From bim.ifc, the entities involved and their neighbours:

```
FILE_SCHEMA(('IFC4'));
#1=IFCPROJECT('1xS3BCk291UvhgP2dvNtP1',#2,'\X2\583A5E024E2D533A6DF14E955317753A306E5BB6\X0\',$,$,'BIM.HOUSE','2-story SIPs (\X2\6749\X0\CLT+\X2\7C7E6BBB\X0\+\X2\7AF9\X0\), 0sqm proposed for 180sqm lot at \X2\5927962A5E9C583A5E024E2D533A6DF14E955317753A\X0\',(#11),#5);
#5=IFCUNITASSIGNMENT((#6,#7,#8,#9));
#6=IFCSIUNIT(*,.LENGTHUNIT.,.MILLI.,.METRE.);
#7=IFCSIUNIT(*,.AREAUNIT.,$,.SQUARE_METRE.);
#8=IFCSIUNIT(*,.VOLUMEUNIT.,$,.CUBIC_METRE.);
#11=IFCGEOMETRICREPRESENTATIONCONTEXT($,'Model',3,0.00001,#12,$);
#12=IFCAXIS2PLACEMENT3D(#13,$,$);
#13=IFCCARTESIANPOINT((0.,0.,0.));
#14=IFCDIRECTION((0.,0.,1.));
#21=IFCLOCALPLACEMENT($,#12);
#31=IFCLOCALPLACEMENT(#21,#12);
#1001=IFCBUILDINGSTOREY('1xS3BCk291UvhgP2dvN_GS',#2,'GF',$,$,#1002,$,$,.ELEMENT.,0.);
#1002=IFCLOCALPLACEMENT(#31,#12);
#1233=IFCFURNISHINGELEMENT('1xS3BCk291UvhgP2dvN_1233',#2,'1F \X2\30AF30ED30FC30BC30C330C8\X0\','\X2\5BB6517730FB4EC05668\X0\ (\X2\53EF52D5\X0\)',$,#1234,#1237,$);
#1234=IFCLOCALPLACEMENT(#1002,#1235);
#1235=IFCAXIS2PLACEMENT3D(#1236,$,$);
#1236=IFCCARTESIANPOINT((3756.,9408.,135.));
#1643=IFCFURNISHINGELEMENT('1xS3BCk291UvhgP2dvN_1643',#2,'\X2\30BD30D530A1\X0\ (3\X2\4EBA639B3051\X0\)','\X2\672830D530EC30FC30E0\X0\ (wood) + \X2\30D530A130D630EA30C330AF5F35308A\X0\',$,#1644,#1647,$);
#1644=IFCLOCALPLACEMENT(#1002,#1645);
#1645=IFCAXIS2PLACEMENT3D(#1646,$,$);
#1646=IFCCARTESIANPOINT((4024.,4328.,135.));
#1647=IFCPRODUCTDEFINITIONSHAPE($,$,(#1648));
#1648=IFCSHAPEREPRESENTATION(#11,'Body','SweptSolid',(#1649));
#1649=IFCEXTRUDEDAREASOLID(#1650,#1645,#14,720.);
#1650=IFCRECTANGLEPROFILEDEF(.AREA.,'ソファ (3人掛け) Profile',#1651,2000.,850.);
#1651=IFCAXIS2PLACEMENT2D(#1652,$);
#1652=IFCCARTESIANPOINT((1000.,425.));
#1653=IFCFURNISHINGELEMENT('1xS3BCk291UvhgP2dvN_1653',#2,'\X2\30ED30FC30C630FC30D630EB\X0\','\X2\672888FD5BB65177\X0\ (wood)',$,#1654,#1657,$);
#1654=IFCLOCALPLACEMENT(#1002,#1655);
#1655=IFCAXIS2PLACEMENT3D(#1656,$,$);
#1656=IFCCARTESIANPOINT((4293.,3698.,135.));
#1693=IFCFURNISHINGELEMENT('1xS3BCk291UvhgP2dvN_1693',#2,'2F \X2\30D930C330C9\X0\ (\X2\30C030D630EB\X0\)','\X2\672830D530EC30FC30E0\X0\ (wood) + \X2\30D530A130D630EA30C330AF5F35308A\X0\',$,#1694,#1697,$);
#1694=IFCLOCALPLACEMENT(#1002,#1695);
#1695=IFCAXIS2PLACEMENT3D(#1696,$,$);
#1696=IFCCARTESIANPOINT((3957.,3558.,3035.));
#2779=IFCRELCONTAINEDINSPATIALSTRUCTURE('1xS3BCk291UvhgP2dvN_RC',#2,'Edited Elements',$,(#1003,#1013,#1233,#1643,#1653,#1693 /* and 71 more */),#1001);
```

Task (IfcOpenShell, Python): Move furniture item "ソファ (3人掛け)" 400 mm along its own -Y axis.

```python
import ifcopenshell
import ifcopenshell.api.geometry
import ifcopenshell.util.placement
import ifcopenshell.util.unit

model = ifcopenshell.open("bim.ifc")
unit_scale = ifcopenshell.util.unit.calculate_unit_scale(model)

item = model.by_guid("1xS3BCk291UvhgP2dvN_1643")
matrix = ifcopenshell.util.placement.get_local_placement(item.ObjectPlacement)
matrix[:3, 3] -= matrix[:3, 1] * 0.4 / unit_scale
ifcopenshell.api.geometry.edit_object_placement(model, product=item, matrix=matrix, is_si=False)

print(ifcopenshell.util.placement.get_local_placement(item.ObjectPlacement).round(3) + 0.0)

model.write("bim_edited.ifc")
```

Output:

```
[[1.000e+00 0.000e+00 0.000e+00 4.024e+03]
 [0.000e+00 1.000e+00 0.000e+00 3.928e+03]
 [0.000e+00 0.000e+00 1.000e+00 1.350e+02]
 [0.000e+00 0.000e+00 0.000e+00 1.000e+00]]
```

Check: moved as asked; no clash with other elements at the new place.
